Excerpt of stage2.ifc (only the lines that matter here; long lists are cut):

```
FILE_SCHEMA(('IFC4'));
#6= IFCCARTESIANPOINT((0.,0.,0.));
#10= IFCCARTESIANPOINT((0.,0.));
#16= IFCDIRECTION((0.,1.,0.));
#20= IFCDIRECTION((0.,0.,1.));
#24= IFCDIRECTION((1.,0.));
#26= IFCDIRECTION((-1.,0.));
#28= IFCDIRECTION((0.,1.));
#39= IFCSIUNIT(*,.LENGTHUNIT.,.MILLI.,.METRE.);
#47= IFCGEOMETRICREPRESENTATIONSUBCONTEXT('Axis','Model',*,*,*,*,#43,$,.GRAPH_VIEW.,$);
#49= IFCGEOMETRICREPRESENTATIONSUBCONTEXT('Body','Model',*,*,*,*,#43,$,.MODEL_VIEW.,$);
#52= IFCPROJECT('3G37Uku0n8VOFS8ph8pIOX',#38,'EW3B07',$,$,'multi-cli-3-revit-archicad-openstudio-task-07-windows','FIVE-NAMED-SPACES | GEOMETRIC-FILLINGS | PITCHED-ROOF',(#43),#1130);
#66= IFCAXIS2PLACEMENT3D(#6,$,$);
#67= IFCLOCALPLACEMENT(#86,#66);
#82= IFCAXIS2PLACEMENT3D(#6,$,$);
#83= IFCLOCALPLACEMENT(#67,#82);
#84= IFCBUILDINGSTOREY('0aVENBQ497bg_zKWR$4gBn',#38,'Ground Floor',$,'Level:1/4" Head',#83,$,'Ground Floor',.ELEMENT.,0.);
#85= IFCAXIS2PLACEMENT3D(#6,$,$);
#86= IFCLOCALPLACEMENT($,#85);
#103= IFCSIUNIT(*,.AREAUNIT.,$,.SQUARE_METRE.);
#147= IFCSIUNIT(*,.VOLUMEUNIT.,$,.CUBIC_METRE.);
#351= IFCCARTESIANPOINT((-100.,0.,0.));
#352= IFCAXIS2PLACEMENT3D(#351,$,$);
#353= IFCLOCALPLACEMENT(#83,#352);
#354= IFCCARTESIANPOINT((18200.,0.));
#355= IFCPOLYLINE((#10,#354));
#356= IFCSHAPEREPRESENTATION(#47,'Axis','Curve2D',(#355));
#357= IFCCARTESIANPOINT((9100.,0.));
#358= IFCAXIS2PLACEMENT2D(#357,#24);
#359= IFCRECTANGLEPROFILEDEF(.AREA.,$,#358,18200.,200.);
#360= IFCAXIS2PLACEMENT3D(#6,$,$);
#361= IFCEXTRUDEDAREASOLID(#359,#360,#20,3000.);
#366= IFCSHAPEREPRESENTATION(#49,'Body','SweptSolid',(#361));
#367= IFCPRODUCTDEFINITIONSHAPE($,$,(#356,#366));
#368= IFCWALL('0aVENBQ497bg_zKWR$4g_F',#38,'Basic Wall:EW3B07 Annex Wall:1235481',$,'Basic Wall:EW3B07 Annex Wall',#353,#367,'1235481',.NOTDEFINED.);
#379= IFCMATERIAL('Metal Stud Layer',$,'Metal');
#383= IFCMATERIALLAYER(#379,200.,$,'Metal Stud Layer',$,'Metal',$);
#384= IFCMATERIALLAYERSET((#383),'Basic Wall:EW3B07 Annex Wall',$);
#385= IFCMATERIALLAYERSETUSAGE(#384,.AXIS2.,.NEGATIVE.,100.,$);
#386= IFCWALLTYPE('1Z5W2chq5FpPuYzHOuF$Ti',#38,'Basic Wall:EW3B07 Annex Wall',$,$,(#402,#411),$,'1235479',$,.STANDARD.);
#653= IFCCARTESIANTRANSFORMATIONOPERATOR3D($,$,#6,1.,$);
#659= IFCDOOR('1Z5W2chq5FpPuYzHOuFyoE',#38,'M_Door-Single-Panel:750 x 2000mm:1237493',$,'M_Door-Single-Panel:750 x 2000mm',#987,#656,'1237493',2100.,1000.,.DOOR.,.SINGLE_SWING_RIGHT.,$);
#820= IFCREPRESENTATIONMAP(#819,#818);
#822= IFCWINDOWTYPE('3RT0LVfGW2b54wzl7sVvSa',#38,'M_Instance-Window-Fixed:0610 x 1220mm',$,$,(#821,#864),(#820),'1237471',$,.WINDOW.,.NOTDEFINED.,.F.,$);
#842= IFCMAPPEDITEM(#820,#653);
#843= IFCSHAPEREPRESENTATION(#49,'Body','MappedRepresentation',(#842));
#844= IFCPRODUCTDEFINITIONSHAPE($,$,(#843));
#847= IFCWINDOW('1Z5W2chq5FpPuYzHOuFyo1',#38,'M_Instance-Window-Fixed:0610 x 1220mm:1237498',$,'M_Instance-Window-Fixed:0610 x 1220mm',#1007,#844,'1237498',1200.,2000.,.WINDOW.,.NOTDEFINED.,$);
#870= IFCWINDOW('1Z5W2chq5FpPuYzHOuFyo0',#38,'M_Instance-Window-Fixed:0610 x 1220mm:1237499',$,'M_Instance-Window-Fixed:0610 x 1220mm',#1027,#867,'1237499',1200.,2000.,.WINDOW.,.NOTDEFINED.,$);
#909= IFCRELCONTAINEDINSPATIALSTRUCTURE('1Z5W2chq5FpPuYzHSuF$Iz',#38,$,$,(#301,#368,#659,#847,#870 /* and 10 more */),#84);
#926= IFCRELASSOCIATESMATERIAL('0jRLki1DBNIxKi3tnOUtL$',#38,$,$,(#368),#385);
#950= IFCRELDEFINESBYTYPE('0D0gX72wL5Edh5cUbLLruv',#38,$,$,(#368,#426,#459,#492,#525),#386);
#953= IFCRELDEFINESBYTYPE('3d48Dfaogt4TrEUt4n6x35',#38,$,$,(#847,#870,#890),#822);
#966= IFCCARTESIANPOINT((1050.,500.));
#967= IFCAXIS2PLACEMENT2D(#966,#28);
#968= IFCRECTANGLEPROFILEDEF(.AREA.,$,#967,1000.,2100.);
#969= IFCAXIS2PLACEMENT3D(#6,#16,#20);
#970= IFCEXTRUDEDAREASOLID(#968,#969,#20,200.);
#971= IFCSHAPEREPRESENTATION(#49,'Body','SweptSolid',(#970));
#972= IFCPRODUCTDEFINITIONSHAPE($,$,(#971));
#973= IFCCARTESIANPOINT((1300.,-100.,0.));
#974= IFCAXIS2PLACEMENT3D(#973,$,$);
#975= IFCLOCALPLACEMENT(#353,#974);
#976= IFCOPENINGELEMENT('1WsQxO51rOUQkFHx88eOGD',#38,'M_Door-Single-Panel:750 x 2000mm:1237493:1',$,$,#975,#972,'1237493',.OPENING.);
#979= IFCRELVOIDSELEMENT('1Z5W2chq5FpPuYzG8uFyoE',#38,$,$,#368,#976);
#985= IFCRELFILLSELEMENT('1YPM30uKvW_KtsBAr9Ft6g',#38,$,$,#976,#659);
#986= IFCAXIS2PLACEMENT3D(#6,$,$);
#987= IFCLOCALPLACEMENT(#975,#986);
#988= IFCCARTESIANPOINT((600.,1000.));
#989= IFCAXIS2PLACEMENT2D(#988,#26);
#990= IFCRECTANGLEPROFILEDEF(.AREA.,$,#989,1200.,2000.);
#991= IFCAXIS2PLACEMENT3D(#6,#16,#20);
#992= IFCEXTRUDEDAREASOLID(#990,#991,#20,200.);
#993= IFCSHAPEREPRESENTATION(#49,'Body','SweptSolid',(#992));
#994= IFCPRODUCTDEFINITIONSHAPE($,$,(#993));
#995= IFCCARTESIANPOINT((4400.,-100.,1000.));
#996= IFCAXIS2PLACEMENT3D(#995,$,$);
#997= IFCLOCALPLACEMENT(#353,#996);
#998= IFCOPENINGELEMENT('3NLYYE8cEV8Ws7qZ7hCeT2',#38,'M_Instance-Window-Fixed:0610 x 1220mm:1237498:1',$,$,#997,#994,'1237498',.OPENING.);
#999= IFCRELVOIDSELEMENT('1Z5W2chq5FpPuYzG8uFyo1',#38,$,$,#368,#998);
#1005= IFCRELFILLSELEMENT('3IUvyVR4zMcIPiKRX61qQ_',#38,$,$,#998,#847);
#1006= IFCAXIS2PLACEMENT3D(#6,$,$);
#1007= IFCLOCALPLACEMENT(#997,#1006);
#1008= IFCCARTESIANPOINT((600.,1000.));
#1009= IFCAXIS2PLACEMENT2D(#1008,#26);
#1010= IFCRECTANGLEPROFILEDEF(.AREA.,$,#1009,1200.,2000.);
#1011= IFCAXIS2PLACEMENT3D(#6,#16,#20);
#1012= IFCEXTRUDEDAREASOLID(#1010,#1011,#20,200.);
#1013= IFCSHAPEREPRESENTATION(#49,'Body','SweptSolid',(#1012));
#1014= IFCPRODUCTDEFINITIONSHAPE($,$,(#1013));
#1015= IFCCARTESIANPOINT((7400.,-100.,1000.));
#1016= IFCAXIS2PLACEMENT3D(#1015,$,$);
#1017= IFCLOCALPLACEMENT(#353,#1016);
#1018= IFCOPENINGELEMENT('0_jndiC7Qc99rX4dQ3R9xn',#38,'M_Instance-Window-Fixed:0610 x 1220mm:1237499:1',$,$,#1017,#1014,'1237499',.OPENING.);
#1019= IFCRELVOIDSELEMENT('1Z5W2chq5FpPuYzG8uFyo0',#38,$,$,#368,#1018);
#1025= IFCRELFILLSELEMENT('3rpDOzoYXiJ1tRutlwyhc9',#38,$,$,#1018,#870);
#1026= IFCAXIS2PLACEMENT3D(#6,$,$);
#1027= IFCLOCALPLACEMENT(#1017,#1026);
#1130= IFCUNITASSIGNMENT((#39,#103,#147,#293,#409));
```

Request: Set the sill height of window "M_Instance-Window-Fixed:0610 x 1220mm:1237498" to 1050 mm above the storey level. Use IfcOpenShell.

```python
import numpy as np
import ifcopenshell
import ifcopenshell.api.geometry
import ifcopenshell.geom
import ifcopenshell.util.element
import ifcopenshell.util.placement
import ifcopenshell.util.shape
import ifcopenshell.util.unit

model = ifcopenshell.open("stage2.ifc")
unit_scale = ifcopenshell.util.unit.calculate_unit_scale(model)

window = model.by_id(847)
opening = window.FillsVoids[0].RelatingOpeningElement
storey = ifcopenshell.util.element.get_container(window, ifc_class="IfcBuildingStorey")
level = ifcopenshell.util.placement.get_local_placement(storey.ObjectPlacement)[2, 3]

# The opening's origin need not be at the sill, so measure its lowest point.
shape = ifcopenshell.geom.create_shape(ifcopenshell.geom.settings(), opening)
bottom = ifcopenshell.util.shape.get_shape_bottom_elevation(shape, shape.geometry) / unit_scale
dz = level + 1.05 / unit_scale - bottom

shift = np.array([0.0, 0.0, dz])
# The window is placed relative to its opening, so it follows when the opening moves.
matrix = ifcopenshell.util.placement.get_local_placement(opening.ObjectPlacement)
matrix[:3, 3] += shift
ifcopenshell.api.geometry.edit_object_placement(
    model, product=opening, matrix=matrix, is_si=False, should_transform_children=True
)

print(f"moved by {dz * unit_scale:+.3f} m")

model.write("stage2-out.ifc")
```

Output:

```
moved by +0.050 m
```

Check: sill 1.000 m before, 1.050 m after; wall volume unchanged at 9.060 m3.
